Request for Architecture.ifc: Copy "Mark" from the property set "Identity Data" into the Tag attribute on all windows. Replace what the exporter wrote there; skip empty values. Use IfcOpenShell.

First a look at what the model holds.

```python
import ifcopenshell
import ifcopenshell.util.element

model = ifcopenshell.open("Architecture.ifc")
print(model.schema)
windows = model.by_type("IfcWindow")
print(len(windows), "windows")
for e in windows[:8]:
    source = ifcopenshell.util.element.get_pset(e, "Identity Data", "Mark")
    target = e.Tag
    print(e.id(), repr(source), repr(target), sep=" | ")
```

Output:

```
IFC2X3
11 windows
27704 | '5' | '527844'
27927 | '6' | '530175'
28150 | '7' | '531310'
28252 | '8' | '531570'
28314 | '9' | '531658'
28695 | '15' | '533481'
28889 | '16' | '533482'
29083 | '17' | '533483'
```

```python
import ifcopenshell
import ifcopenshell.util.element

model = ifcopenshell.open("Architecture.ifc")

count = 0
for e in model.by_type("IfcWindow"):
    value = ifcopenshell.util.element.get_pset(e, "Identity Data", "Mark")
    current = e.Tag
    if not value or not value.strip() or current == value:
        continue
    e.Tag = value
    count += 1

print(count, "windows updated")

model.write("Architecture_rev.ifc")
```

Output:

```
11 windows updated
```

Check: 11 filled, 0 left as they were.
